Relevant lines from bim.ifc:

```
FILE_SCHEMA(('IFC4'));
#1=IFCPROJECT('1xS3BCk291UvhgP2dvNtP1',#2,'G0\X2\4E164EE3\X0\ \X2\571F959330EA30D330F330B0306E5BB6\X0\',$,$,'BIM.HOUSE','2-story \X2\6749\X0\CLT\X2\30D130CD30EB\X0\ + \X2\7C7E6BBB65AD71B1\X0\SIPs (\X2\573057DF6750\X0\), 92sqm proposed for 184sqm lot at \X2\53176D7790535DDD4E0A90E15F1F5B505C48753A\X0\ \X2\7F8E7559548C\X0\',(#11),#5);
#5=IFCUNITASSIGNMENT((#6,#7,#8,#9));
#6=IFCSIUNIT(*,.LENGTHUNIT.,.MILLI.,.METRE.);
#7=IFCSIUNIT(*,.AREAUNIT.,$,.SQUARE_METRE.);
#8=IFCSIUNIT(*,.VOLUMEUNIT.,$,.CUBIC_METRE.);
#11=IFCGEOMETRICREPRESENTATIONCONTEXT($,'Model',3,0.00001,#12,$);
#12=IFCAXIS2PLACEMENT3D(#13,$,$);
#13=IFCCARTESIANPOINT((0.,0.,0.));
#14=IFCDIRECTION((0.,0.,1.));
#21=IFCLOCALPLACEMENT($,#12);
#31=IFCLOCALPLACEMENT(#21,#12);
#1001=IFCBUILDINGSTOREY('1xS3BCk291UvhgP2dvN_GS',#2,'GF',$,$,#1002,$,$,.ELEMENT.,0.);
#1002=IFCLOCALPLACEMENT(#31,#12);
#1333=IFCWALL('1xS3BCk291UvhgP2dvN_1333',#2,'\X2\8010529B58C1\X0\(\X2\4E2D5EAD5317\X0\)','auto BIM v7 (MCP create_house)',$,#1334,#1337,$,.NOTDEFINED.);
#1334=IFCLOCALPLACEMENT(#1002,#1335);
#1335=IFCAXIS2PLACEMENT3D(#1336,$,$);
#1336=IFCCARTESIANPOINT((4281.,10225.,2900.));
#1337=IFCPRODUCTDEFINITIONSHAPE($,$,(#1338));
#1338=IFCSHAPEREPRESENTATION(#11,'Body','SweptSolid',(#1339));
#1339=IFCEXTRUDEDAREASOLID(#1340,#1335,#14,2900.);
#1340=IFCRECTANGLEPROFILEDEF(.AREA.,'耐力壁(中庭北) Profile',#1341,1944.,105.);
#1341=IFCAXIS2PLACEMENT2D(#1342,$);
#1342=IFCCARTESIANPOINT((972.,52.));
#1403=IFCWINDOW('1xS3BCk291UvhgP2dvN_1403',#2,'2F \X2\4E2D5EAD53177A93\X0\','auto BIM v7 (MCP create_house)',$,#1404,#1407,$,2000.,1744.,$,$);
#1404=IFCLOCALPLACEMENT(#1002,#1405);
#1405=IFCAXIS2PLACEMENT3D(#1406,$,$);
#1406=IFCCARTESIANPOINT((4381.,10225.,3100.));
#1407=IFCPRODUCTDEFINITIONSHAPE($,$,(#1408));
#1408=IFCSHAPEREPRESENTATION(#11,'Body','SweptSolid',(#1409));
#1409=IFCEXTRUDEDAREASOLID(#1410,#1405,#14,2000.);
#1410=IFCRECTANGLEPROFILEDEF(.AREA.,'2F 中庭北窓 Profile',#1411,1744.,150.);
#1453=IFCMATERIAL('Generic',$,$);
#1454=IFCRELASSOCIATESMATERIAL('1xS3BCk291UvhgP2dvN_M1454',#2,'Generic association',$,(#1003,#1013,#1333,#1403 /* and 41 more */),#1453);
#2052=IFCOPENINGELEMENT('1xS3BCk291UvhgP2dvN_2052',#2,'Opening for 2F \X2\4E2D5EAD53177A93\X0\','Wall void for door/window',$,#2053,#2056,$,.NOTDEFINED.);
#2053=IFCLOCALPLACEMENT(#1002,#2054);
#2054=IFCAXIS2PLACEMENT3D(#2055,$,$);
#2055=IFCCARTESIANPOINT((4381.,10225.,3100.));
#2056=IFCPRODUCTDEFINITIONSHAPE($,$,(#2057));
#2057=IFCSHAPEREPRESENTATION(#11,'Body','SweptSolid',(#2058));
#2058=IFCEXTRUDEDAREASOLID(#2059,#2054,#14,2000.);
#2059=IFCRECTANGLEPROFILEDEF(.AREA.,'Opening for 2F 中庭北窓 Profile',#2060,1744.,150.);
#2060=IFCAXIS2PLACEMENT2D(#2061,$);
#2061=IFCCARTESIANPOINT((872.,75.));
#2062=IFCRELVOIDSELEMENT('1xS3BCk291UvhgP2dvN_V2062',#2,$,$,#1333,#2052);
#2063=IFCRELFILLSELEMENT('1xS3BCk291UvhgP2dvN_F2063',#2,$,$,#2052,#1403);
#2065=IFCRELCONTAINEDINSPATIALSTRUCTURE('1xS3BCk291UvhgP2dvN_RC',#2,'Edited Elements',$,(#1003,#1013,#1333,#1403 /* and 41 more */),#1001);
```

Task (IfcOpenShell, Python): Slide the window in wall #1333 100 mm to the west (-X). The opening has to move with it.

```python
import ifcopenshell
import ifcopenshell.api.geometry
import ifcopenshell.util.placement

model = ifcopenshell.open("bim.ifc")

window = model.by_id(1403)
opening = window.FillsVoids[0].RelatingOpeningElement
wall = opening.VoidsElements[0].RelatingBuildingElement

wall_matrix = ifcopenshell.util.placement.get_local_placement(wall.ObjectPlacement)
shift = wall_matrix[:3, 0] * -100.0
before = ifcopenshell.util.placement.get_local_placement(window.ObjectPlacement)[:3, 3].copy()

# The window is not placed relative to its opening, so move both.
for product in (opening, window):
    matrix = ifcopenshell.util.placement.get_local_placement(product.ObjectPlacement)
    matrix[:3, 3] += shift
    ifcopenshell.api.geometry.edit_object_placement(model, product=product, matrix=matrix, is_si=False)

after = ifcopenshell.util.placement.get_local_placement(window.ObjectPlacement)[:3, 3]
print("window moved by", (after - before).round(3) + 0.0)

model.write("bim-out.ifc")
```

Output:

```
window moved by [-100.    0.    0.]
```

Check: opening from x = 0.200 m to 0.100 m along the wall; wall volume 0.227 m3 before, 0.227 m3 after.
